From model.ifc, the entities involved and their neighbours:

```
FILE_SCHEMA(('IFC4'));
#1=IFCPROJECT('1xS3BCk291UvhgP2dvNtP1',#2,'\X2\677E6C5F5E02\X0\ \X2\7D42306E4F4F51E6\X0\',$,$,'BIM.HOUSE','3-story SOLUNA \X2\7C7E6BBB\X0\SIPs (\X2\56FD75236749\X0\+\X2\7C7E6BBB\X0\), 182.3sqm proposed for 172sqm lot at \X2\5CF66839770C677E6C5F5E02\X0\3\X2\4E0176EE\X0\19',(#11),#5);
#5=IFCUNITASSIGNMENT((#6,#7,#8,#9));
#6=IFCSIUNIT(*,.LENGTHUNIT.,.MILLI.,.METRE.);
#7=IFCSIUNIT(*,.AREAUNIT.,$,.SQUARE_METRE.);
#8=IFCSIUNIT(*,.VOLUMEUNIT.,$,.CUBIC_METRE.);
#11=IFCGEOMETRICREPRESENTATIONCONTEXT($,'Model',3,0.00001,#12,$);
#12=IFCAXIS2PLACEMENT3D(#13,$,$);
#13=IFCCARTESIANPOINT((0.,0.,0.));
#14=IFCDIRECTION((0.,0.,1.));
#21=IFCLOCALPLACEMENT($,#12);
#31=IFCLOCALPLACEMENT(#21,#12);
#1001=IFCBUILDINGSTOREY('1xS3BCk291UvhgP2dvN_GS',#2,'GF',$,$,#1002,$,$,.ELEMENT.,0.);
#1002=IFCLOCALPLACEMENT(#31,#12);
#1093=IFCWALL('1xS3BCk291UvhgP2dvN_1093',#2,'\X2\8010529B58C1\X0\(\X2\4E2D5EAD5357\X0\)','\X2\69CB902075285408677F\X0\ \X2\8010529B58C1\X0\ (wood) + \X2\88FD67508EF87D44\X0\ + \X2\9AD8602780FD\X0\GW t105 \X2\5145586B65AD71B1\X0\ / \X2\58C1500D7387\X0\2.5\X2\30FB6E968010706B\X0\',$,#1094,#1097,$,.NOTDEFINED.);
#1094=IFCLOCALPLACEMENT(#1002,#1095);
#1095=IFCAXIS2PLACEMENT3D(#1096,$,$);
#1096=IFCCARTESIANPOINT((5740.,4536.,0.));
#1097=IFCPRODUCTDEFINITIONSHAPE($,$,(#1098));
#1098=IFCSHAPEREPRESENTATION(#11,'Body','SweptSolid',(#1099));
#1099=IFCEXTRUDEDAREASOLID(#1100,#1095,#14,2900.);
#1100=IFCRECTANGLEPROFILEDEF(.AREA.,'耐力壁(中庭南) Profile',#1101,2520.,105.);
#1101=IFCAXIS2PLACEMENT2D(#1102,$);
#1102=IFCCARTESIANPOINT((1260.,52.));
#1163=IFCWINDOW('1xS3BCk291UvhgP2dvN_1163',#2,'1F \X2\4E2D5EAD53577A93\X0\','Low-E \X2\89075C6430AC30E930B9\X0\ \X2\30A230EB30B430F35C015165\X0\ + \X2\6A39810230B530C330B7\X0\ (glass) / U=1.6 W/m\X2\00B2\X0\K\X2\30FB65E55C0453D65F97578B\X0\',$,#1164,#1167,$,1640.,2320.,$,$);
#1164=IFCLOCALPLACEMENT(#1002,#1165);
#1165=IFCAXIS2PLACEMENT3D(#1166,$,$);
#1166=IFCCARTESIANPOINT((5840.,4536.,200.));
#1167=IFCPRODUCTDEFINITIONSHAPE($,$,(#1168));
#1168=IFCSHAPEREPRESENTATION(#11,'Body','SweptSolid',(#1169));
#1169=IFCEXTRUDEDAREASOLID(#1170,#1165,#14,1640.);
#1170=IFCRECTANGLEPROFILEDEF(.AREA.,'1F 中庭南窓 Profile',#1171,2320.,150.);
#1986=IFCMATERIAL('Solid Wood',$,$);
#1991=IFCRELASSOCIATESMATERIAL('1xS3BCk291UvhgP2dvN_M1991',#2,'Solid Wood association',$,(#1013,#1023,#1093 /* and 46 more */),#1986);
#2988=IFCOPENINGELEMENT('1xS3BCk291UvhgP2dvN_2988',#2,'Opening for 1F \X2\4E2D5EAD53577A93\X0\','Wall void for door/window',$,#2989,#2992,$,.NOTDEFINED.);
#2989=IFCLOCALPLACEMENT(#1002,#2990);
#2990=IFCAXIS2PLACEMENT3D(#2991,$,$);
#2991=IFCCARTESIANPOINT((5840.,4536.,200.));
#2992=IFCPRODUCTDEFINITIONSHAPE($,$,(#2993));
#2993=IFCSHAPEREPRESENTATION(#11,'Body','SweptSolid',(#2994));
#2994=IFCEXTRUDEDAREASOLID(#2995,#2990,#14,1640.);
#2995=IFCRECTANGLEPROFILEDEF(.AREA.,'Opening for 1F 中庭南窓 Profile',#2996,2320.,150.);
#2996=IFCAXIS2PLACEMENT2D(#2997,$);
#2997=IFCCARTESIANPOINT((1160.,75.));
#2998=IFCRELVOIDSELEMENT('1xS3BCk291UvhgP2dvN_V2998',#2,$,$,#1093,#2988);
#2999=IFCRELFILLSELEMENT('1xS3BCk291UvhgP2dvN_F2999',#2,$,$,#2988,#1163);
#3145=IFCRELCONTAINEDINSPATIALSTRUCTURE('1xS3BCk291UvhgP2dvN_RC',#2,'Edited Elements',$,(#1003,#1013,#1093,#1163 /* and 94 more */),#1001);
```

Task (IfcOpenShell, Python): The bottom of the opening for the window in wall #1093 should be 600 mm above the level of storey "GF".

```python
import numpy as np
import ifcopenshell
import ifcopenshell.api.geometry
import ifcopenshell.geom
import ifcopenshell.util.element
import ifcopenshell.util.placement
import ifcopenshell.util.shape
import ifcopenshell.util.unit

model = ifcopenshell.open("model.ifc")
unit_scale = ifcopenshell.util.unit.calculate_unit_scale(model)

window = model.by_guid("1xS3BCk291UvhgP2dvN_1163")
opening = window.FillsVoids[0].RelatingOpeningElement
storey = ifcopenshell.util.element.get_container(window, ifc_class="IfcBuildingStorey")
level = ifcopenshell.util.placement.get_local_placement(storey.ObjectPlacement)[2, 3]

# The opening's origin need not be at the sill, so measure its lowest point.
shape = ifcopenshell.geom.create_shape(ifcopenshell.geom.settings(), opening)
bottom = ifcopenshell.util.shape.get_shape_bottom_elevation(shape, shape.geometry) / unit_scale
dz = level + 600.0 - bottom

shift = np.array([0.0, 0.0, dz])
# The window is not placed relative to its opening, so move both.
for product in (opening, window):
    matrix = ifcopenshell.util.placement.get_local_placement(product.ObjectPlacement)
    matrix[:3, 3] += shift
    ifcopenshell.api.geometry.edit_object_placement(model, product=product, matrix=matrix, is_si=False)

print(f"moved by {dz * unit_scale:+.3f} m")

model.write("model_edited.ifc")
```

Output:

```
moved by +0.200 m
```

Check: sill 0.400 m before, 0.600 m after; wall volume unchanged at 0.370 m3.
